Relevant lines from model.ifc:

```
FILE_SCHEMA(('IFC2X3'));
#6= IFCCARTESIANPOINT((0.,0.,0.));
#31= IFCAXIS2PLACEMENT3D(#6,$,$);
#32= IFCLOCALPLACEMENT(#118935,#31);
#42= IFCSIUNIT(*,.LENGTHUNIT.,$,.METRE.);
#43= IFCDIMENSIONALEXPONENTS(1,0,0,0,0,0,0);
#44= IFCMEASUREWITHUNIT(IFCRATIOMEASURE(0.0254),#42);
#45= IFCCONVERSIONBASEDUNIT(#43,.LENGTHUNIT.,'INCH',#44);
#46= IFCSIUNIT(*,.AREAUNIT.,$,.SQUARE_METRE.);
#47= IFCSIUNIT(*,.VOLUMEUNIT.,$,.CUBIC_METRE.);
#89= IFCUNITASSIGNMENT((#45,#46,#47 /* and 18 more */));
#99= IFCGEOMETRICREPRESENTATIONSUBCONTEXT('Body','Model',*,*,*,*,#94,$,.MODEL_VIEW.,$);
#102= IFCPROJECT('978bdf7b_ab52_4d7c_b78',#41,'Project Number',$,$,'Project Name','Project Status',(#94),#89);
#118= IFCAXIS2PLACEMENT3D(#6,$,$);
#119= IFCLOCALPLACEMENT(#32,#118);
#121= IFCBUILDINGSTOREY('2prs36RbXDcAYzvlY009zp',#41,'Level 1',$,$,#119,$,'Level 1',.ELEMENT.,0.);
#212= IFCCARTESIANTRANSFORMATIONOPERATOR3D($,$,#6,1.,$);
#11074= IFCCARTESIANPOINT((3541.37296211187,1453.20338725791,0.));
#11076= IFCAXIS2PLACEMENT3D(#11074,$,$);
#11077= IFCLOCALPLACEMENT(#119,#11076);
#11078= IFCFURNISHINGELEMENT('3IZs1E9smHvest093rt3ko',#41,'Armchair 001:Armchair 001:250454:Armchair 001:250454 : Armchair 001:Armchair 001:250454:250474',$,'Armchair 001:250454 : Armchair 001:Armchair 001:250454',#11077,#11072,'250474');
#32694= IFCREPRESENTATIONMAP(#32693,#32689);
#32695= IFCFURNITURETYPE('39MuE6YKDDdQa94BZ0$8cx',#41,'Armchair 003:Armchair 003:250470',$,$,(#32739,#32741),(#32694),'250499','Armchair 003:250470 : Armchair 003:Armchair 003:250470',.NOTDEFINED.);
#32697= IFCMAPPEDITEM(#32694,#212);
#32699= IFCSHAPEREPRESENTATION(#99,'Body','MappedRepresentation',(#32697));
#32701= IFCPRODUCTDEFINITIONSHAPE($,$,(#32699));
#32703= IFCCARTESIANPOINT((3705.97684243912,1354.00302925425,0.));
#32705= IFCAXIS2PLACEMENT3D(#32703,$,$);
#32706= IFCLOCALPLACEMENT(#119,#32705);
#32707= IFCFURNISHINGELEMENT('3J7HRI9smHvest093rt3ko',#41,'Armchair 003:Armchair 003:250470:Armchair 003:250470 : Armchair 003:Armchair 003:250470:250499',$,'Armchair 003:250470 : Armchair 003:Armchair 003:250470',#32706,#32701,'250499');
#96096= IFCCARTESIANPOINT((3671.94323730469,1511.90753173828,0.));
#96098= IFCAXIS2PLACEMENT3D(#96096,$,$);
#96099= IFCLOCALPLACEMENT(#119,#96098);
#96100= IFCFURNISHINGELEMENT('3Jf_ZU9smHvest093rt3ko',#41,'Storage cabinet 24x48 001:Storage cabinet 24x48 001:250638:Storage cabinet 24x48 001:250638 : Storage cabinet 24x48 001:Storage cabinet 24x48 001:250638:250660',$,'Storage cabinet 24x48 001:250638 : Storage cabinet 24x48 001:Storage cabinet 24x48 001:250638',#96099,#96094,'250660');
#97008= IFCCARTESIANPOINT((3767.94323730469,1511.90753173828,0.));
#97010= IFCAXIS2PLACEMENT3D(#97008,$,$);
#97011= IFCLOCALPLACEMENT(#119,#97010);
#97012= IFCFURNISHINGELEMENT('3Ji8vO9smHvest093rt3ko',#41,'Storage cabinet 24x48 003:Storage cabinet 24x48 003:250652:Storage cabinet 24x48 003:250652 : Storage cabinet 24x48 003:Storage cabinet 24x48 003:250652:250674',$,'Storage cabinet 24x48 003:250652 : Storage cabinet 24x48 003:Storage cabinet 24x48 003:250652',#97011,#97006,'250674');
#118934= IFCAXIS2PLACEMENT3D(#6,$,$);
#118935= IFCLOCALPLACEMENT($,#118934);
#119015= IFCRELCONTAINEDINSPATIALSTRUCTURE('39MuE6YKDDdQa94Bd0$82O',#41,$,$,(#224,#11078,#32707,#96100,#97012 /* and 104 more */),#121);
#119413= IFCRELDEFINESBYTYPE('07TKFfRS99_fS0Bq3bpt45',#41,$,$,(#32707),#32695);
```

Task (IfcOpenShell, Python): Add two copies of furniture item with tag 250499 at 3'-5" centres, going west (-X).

```python
import numpy as np
import ifcopenshell
import ifcopenshell.api.geometry
import ifcopenshell.api.root
import ifcopenshell.util.element
import ifcopenshell.util.placement
import ifcopenshell.util.unit

model = ifcopenshell.open("model.ifc")
unit_scale = ifcopenshell.util.unit.calculate_unit_scale(model)


def reuse_history(source, copy):
    """copy_class also copies each property set's owner history, people and application; keep the originals."""
    for rel in copy.IsDefinedBy:
        if rel.is_a("IfcRelDefinesByProperties") and (history := rel.RelatingPropertyDefinition.OwnerHistory):
            rel.RelatingPropertyDefinition.OwnerHistory = source.OwnerHistory
            ifcopenshell.util.element.remove_deep2(model, history)


source = model.by_guid("3J7HRI9smHvest093rt3ko")
base = ifcopenshell.util.placement.get_local_placement(source.ObjectPlacement)
step = np.array([-1.0, 0.0, 0.0]) * 41 * 0.0254 / unit_scale

for i in range(1, 3):
    copy = ifcopenshell.api.root.copy_class(model, product=source)
    copy.Representation = ifcopenshell.util.element.copy_deep(
        model, source.Representation, exclude=["IfcGeometricRepresentationContext", "IfcRepresentationMap"]
    )
    copy.Name = "Armchair 003:Armchair 003:250470:Armchair 003:250470 : Armchair 003:Armchair 003"
    copy.Tag = None
    reuse_history(source, copy)
    matrix = base.copy()
    matrix[:3, 3] += i * step
    print("added at", matrix[:3, 3].round(3) + 0.0)
    ifcopenshell.api.geometry.edit_object_placement(model, product=copy, matrix=matrix, is_si=False)

model.write("model-out.ifc")
```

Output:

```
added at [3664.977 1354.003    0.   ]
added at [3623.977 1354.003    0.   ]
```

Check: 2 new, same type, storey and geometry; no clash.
